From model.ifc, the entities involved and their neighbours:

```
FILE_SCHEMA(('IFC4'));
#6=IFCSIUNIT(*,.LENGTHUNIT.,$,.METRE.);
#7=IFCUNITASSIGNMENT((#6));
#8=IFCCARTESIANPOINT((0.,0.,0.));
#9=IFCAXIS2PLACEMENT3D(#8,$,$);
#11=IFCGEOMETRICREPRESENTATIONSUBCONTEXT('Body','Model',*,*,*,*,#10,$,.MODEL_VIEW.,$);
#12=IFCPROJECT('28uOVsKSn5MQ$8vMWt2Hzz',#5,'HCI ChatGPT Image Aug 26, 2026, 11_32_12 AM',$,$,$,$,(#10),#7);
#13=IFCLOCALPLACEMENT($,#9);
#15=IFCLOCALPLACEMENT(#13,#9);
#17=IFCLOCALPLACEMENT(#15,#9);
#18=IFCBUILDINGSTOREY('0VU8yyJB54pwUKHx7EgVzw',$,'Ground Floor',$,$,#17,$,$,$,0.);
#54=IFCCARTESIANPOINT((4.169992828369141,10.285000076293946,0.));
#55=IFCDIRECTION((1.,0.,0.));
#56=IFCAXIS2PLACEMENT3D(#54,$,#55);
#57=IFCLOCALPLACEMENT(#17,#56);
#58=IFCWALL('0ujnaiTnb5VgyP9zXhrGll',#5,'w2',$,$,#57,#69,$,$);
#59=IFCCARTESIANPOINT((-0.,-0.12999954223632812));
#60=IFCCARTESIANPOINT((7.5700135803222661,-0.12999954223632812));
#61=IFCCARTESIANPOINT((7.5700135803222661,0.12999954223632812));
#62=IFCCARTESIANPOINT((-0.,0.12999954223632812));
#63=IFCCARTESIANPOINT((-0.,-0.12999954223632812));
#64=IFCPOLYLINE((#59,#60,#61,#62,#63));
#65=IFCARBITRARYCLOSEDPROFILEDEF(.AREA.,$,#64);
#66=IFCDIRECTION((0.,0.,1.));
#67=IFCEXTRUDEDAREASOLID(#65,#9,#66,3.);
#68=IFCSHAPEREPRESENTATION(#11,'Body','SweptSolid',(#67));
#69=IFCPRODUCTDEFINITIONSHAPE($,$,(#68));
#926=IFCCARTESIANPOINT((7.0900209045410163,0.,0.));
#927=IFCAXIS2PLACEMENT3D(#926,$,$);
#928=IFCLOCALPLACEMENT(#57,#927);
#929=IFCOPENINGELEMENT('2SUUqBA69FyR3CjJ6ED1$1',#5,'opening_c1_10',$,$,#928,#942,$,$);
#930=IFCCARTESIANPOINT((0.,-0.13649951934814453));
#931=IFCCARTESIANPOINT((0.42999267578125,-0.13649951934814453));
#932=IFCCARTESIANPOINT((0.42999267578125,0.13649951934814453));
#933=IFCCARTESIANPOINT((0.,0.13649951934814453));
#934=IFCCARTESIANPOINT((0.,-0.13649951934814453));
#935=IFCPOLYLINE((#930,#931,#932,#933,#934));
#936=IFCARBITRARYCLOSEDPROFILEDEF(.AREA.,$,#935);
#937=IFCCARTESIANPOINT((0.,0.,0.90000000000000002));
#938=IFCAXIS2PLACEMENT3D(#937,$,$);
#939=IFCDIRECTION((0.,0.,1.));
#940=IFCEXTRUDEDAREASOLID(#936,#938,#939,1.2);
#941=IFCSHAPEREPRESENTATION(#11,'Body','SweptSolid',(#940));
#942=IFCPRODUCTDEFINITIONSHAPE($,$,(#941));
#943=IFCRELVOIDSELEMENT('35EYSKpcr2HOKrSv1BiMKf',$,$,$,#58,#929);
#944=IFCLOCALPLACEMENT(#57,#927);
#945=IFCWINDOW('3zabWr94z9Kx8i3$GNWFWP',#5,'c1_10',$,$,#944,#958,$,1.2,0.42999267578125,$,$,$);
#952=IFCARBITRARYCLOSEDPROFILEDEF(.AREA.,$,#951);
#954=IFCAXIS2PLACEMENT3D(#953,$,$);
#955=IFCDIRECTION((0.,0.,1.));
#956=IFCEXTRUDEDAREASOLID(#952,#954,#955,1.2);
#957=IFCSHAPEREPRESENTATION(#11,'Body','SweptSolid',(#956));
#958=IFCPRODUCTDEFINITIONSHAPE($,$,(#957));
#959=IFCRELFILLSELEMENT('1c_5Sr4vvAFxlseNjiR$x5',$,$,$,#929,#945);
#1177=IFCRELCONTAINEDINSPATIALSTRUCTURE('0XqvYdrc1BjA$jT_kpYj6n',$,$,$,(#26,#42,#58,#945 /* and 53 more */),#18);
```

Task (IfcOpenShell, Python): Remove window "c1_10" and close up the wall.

```python
import ifcopenshell
import ifcopenshell.api.feature
import ifcopenshell.api.root
import ifcopenshell.geom
import ifcopenshell.util.shape

model = ifcopenshell.open("model.ifc")
settings = ifcopenshell.geom.settings()


def volume(element):
    """Net volume in cubic metres, openings subtracted."""
    shape = ifcopenshell.geom.create_shape(settings, element)
    return ifcopenshell.util.shape.get_volume(shape.geometry)


window = model.by_guid("3zabWr94z9Kx8i3$GNWFWP")
opening = window.FillsVoids[0].RelatingOpeningElement
wall = opening.VoidsElements[0].RelatingBuildingElement
before = volume(wall)

ifcopenshell.api.root.remove_product(model, product=window)
ifcopenshell.api.feature.remove_feature(model, feature=opening)

after = volume(wall)

print(f"wall volume {before:.3f} -> {after:.3f} m3")

model.write("model-out.ifc")
```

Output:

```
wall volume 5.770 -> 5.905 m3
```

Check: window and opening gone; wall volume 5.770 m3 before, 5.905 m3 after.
